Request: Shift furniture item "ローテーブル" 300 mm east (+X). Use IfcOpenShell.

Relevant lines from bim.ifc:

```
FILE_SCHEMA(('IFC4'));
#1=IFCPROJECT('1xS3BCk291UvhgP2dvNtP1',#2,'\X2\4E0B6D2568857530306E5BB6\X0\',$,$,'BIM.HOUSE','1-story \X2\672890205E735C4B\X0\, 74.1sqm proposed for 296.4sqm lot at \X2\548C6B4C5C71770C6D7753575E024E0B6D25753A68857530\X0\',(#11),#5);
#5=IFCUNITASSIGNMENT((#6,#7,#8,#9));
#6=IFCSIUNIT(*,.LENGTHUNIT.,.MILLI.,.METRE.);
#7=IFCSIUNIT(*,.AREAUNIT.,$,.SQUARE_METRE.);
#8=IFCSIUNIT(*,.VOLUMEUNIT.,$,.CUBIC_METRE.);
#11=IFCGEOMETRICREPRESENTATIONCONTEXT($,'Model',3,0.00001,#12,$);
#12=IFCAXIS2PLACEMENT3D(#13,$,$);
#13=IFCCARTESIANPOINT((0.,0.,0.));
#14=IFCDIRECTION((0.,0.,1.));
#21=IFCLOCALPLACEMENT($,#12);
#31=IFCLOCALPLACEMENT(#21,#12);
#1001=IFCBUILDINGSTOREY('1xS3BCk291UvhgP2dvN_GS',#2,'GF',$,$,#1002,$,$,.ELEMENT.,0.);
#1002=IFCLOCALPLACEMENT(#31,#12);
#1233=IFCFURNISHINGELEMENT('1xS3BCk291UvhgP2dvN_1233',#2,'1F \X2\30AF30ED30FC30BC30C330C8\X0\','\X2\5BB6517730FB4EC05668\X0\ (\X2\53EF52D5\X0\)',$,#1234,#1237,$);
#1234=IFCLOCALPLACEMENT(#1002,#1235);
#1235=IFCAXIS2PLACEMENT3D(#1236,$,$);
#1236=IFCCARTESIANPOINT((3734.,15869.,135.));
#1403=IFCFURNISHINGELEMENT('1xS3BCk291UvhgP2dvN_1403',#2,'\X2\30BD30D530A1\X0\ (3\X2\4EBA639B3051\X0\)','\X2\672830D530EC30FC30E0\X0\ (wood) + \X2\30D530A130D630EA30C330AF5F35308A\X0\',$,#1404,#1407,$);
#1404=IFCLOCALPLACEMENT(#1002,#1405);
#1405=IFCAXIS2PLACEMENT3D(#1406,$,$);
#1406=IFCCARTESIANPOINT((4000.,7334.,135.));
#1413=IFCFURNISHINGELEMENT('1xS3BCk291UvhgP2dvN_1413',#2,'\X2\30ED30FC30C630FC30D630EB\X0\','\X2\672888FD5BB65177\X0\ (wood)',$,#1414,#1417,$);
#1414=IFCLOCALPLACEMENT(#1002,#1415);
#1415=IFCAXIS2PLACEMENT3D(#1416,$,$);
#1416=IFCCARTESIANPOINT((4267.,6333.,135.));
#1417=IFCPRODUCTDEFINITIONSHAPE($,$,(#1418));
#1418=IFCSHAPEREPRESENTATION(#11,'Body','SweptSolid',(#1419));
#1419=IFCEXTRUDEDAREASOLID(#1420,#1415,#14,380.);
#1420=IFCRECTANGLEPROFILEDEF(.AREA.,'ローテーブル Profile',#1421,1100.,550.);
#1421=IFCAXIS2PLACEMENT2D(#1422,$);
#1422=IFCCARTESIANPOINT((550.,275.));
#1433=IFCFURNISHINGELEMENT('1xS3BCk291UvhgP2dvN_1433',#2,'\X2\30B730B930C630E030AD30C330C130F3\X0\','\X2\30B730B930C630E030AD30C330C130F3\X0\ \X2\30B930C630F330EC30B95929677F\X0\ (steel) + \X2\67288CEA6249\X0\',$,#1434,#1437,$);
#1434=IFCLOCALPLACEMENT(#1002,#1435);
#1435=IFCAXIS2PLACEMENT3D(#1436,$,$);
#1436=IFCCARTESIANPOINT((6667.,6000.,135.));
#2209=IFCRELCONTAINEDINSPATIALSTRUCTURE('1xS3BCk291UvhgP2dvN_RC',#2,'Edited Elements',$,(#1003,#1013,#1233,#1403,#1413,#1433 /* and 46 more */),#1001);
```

```python
import ifcopenshell
import ifcopenshell.api.geometry
import ifcopenshell.util.placement
import ifcopenshell.util.unit

model = ifcopenshell.open("bim.ifc")
unit_scale = ifcopenshell.util.unit.calculate_unit_scale(model)

item = model.by_guid("1xS3BCk291UvhgP2dvN_1413")
matrix = ifcopenshell.util.placement.get_local_placement(item.ObjectPlacement)
matrix[0, 3] += 0.3 / unit_scale
ifcopenshell.api.geometry.edit_object_placement(model, product=item, matrix=matrix, is_si=False)

print(ifcopenshell.util.placement.get_local_placement(item.ObjectPlacement).round(3) + 0.0)

model.write("bim_v2.ifc")
```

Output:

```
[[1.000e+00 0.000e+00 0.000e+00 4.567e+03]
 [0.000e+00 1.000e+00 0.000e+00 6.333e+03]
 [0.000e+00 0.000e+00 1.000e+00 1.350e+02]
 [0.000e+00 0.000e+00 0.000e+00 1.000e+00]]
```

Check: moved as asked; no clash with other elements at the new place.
